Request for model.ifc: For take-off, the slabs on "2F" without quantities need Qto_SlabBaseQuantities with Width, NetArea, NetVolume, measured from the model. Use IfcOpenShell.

First a look at what the model holds.

```python
import ifcopenshell
import ifcopenshell.util.element
import ifcopenshell.util.unit

model = ifcopenshell.open("model.ifc")
print(model.schema)
for unit_type in ("LENGTHUNIT", "AREAUNIT", "VOLUMEUNIT"):
    print(unit_type, ifcopenshell.util.unit.calculate_unit_scale(model, unit_type))
storey = next(s for s in model.by_type("IfcBuildingStorey") if s.Name == "2F")
slabs = [e for e in ifcopenshell.util.element.get_decomposition(storey) if e.is_a("IfcSlab")]
for e in sorted(slabs, key=lambda e: e.id()):
    print(e.id(), e.is_a(), e.Name, list(ifcopenshell.util.element.get_psets(e, qtos_only=True)), sep=" | ")
```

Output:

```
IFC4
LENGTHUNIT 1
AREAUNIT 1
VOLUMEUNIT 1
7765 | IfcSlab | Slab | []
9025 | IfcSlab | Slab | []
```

```python
import ifcopenshell
import ifcopenshell.api.pset
import ifcopenshell.geom
import ifcopenshell.util.element
import ifcopenshell.util.shape
import ifcopenshell.util.unit

model = ifcopenshell.open("model.ifc")
unit_scale = ifcopenshell.util.unit.calculate_unit_scale(model)
area_scale = ifcopenshell.util.unit.calculate_unit_scale(model, "AREAUNIT")
volume_scale = ifcopenshell.util.unit.calculate_unit_scale(model, "VOLUMEUNIT")
settings = ifcopenshell.geom.settings()

storey = next(s for s in model.by_type("IfcBuildingStorey") if s.Name == "2F")
slabs = [e for e in ifcopenshell.util.element.get_decomposition(storey) if e.is_a("IfcSlab")]

for e in sorted(slabs, key=lambda e: e.id()):
    if ifcopenshell.util.element.get_psets(e, qtos_only=True, should_inherit=False):
        continue
    # Geometry comes back in metres, in the element's own axes.
    shape = ifcopenshell.geom.create_shape(settings, e)
    values = {
        "Width": ifcopenshell.util.shape.get_z(shape.geometry) / unit_scale,
        "NetArea": ifcopenshell.util.shape.get_footprint_area(shape.geometry) / area_scale,
        "NetVolume": ifcopenshell.util.shape.get_volume(shape.geometry) / volume_scale,
    }
    qto = ifcopenshell.api.pset.add_qto(model, product=e, name="Qto_SlabBaseQuantities")
    ifcopenshell.api.pset.edit_qto(model, qto=qto, properties=values)
    print(e.id(), {k: round(v, 3) for k, v in values.items()})

model.write("model_v2.ifc")
```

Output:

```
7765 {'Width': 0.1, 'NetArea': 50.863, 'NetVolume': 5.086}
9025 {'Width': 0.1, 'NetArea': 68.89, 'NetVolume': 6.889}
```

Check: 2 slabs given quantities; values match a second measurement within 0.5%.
